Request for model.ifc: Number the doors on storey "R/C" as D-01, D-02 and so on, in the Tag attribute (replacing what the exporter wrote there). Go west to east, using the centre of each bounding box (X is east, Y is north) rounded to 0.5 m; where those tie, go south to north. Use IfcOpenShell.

First a look at what the model holds.

```python
import ifcopenshell
import ifcopenshell.util.element
import ifcopenshell.util.placement

model = ifcopenshell.open("model.ifc")
print(model.schema)
storey = next(s for s in model.by_type("IfcBuildingStorey") if s.Name == "R/C")
doors = [e for e in ifcopenshell.util.element.get_decomposition(storey) if e.is_a("IfcDoor")]
for e in sorted(doors, key=lambda e: e.id()):
    origin = ifcopenshell.util.placement.get_local_placement(e.ObjectPlacement)[:3, 3]
    print(e.id(), e.Tag, e.Name, origin.round(2) + 0.0, sep=" | ")
```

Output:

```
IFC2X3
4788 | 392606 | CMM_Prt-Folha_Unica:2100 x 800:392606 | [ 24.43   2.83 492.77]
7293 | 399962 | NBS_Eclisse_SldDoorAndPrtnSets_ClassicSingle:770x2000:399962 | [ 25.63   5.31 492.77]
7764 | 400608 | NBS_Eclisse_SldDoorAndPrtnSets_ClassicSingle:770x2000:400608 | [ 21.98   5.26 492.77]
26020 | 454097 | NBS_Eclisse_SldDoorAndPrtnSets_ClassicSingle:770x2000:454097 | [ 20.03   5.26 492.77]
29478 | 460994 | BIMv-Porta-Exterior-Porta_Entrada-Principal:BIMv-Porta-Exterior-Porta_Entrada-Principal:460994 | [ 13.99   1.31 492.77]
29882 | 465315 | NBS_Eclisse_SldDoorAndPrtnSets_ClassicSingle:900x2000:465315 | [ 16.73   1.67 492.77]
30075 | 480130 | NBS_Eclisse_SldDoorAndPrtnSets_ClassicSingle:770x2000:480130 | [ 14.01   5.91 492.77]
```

```python
import ifcopenshell
import ifcopenshell.geom
import ifcopenshell.util.element
import ifcopenshell.util.shape

model = ifcopenshell.open("model.ifc")
settings = ifcopenshell.geom.settings()
settings.set("use-world-coords", True)


def centre(element):
    shape = ifcopenshell.geom.create_shape(settings, element)
    return ifcopenshell.util.shape.get_bbox_centroid(shape.geometry)


storey = next(s for s in model.by_type("IfcBuildingStorey") if s.Name == "R/C")
doors = [e for e in ifcopenshell.util.element.get_decomposition(storey) if e.is_a("IfcDoor")]

# Insertion points can sit at a corner or the storey origin, so sort by the geometry (in metres).
centres = {e: centre(e) for e in doors}
doors.sort(key=lambda e: (round(centres[e][0] / 0.5), centres[e][1]))

for i, e in enumerate(doors, start=1):
    number = f"D-{i:02d}"
    e.Tag = number
    print(e.id(), number)

model.write("model_rev.ifc")
```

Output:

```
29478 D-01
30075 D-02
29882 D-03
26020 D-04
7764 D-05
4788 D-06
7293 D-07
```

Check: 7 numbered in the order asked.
